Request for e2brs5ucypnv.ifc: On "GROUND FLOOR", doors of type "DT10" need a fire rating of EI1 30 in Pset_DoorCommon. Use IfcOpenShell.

First a look at what the model holds.

```python
import ifcopenshell
import ifcopenshell.util.element

model = ifcopenshell.open("e2brs5ucypnv.ifc")
print(model.schema)
storey = next(s for s in model.by_type("IfcBuildingStorey") if s.Name == "GROUND FLOOR")
doors = [e for e in ifcopenshell.util.element.get_decomposition(storey) if e.is_a("IfcDoor")]
seen = {}
for e in doors:
    element_type = ifcopenshell.util.element.get_type(e)
    key = (element_type.Name if element_type != e and element_type else None, ifcopenshell.util.element.get_pset(e, "Pset_DoorCommon", "FireRating"))
    seen[key] = seen.get(key, 0) + 1
for (name, value), count in sorted(seen.items(), key=str):
    print(count, "x", name, "|", value)
```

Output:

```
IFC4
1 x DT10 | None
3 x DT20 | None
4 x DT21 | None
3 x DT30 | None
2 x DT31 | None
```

```python
import ifcopenshell
import ifcopenshell.api.pset
import ifcopenshell.util.element

model = ifcopenshell.open("e2brs5ucypnv.ifc")

storey = next(s for s in model.by_type("IfcBuildingStorey") if s.Name == "GROUND FLOOR")
doors = [e for e in ifcopenshell.util.element.get_decomposition(storey) if e.is_a("IfcDoor")]

count = 0
for e in doors:
    element_type = ifcopenshell.util.element.get_type(e)
    if element_type in (None, e) or element_type.Name != "DT10":
        continue
    # add_pset returns the element's existing set when there is one.
    pset = ifcopenshell.api.pset.add_pset(model, product=e, name="Pset_DoorCommon")
    ifcopenshell.api.pset.edit_pset(model, pset=pset, properties={"FireRating": "EI1 30"})
    count += 1

print(count, "doors updated")

model.write("e2brs5ucypnv_v2.ifc")
```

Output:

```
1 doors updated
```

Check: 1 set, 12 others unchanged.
